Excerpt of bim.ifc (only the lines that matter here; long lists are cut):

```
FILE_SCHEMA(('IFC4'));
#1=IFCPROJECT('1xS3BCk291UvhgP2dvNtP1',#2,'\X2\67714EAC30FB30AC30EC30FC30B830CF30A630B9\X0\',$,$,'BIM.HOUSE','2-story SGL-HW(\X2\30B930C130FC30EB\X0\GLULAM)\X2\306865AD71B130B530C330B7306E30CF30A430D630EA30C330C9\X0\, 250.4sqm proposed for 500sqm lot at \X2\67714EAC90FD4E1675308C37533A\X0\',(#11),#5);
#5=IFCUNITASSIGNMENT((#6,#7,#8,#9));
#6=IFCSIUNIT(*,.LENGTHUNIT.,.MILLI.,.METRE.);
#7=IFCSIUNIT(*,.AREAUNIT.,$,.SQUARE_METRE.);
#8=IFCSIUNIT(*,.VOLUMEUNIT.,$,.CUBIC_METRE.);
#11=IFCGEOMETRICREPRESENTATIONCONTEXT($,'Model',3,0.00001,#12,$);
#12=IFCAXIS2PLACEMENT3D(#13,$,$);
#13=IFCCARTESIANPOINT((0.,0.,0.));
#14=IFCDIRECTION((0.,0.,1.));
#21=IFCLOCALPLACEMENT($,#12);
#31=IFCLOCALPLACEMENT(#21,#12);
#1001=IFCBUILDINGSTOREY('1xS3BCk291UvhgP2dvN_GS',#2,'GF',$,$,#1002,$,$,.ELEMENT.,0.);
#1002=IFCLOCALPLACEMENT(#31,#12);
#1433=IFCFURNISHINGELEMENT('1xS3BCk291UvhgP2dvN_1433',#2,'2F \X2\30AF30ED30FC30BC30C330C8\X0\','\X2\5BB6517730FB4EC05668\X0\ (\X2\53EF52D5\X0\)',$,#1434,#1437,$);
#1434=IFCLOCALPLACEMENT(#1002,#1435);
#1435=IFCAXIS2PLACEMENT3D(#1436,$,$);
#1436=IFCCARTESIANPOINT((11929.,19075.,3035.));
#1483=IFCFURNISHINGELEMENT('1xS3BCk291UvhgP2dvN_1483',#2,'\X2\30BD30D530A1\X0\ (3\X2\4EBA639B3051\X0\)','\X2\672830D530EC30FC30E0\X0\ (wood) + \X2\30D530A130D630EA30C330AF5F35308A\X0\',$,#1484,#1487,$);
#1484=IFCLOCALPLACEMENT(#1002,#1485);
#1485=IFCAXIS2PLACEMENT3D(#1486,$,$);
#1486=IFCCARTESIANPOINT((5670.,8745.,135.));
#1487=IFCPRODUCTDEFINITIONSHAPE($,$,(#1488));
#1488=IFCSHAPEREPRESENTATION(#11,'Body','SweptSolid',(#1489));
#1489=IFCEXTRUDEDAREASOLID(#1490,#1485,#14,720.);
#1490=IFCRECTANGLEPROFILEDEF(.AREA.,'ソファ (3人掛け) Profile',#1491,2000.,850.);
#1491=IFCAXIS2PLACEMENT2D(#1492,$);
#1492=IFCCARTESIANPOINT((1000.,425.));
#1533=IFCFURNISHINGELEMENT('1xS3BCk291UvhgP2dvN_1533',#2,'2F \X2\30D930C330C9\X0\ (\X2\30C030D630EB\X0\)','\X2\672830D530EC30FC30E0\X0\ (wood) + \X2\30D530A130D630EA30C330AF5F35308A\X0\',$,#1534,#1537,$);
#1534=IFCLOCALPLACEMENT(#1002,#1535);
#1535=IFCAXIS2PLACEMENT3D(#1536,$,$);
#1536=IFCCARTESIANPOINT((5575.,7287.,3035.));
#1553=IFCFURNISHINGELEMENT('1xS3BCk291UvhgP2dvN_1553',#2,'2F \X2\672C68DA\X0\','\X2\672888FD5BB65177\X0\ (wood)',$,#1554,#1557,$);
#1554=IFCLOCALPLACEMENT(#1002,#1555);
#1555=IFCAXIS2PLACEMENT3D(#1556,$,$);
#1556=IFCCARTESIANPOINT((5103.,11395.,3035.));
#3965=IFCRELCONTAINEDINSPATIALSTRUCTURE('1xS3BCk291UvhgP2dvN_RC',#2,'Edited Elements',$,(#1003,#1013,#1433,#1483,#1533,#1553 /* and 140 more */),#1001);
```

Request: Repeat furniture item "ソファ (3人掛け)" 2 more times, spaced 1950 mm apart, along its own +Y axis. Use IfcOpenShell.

```python
import ifcopenshell
import ifcopenshell.api.geometry
import ifcopenshell.api.root
import ifcopenshell.util.element
import ifcopenshell.util.placement
import ifcopenshell.util.unit

model = ifcopenshell.open("bim.ifc")
unit_scale = ifcopenshell.util.unit.calculate_unit_scale(model)


def reuse_history(source, copy):
    """copy_class also copies each property set's owner history, people and application; keep the originals."""
    for rel in copy.IsDefinedBy:
        if rel.is_a("IfcRelDefinesByProperties") and (history := rel.RelatingPropertyDefinition.OwnerHistory):
            rel.RelatingPropertyDefinition.OwnerHistory = source.OwnerHistory
            ifcopenshell.util.element.remove_deep2(model, history)


source = model.by_guid("1xS3BCk291UvhgP2dvN_1483")
base = ifcopenshell.util.placement.get_local_placement(source.ObjectPlacement)
step = base[:3, 1] * 1.95 / unit_scale

for i in range(1, 3):
    copy = ifcopenshell.api.root.copy_class(model, product=source)
    copy.Representation = ifcopenshell.util.element.copy_deep(
        model, source.Representation, exclude=["IfcGeometricRepresentationContext", "IfcRepresentationMap"]
    )
    reuse_history(source, copy)
    matrix = base.copy()
    matrix[:3, 3] += i * step
    print("added at", matrix[:3, 3].round(3) + 0.0)
    ifcopenshell.api.geometry.edit_object_placement(model, product=copy, matrix=matrix, is_si=False)

model.write("bim_updated.ifc")
```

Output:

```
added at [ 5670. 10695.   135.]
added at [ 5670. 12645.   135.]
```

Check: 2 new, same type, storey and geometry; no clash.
